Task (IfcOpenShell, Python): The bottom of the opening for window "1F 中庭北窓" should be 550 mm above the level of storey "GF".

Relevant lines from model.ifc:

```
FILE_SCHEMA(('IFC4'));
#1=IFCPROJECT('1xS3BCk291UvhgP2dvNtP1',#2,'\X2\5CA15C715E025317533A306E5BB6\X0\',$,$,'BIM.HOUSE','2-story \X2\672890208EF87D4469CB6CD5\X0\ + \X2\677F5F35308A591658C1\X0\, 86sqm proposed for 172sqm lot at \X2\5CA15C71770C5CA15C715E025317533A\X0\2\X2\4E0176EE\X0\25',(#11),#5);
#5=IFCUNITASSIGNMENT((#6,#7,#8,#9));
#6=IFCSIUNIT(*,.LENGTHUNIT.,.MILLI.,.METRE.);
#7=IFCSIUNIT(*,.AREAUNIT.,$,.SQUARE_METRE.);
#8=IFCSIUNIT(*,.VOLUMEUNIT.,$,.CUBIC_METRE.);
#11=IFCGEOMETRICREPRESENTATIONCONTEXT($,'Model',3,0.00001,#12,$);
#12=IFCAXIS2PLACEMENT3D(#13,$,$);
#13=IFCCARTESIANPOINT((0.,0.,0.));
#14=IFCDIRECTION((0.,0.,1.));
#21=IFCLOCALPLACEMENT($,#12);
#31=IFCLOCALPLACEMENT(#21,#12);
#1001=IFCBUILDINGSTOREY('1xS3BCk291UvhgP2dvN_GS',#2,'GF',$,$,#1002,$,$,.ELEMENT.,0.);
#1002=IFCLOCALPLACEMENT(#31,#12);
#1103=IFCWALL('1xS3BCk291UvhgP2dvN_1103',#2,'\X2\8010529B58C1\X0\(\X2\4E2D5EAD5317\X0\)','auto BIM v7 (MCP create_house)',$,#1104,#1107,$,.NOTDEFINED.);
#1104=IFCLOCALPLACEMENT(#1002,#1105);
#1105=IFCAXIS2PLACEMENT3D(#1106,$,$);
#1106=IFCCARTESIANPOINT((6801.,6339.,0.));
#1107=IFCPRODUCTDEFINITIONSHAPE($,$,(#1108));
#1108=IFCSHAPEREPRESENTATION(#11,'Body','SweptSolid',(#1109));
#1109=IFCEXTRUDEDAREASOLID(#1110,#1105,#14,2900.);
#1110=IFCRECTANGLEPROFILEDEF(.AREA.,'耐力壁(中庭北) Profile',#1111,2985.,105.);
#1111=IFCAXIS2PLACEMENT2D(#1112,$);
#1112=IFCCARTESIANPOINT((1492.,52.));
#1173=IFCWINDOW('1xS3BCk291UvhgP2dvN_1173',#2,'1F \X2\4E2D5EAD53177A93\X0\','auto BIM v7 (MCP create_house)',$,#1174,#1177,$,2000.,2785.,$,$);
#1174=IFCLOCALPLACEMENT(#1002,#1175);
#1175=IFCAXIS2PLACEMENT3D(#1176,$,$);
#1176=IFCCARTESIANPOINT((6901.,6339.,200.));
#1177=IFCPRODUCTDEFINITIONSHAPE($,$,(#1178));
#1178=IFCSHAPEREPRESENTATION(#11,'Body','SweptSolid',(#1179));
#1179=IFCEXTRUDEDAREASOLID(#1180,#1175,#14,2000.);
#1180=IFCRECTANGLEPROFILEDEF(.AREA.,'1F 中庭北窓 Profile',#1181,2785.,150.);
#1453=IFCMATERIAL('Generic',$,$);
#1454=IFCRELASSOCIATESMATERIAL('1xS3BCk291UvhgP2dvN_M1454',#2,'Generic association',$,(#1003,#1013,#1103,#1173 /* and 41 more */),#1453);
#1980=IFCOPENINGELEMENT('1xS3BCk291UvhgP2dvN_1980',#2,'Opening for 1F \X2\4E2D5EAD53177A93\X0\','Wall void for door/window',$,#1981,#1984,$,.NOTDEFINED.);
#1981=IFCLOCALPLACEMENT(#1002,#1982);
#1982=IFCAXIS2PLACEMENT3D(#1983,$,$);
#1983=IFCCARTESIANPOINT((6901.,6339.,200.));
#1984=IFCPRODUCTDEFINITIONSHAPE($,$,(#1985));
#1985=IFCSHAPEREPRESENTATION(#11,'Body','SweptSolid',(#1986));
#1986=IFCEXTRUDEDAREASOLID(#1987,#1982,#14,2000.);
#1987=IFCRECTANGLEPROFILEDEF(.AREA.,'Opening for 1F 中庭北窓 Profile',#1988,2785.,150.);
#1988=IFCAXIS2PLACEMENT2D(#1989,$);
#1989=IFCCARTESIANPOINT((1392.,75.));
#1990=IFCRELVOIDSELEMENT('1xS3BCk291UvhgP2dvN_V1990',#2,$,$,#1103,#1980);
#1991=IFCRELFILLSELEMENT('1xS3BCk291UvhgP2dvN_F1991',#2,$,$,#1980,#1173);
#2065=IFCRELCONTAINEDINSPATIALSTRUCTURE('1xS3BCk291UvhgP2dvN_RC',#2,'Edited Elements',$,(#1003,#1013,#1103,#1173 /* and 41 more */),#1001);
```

```python
import numpy as np
import ifcopenshell
import ifcopenshell.api.geometry
import ifcopenshell.geom
import ifcopenshell.util.element
import ifcopenshell.util.placement
import ifcopenshell.util.shape
import ifcopenshell.util.unit

model = ifcopenshell.open("model.ifc")
unit_scale = ifcopenshell.util.unit.calculate_unit_scale(model)

window = model.by_guid("1xS3BCk291UvhgP2dvN_1173")
opening = window.FillsVoids[0].RelatingOpeningElement
storey = ifcopenshell.util.element.get_container(window, ifc_class="IfcBuildingStorey")
level = ifcopenshell.util.placement.get_local_placement(storey.ObjectPlacement)[2, 3]

# The opening's origin need not be at the sill, so measure its lowest point.
shape = ifcopenshell.geom.create_shape(ifcopenshell.geom.settings(), opening)
bottom = ifcopenshell.util.shape.get_shape_bottom_elevation(shape, shape.geometry) / unit_scale
dz = level + 0.55 / unit_scale - bottom

shift = np.array([0.0, 0.0, dz])
# The window is not placed relative to its opening, so move both.
for product in (opening, window):
    matrix = ifcopenshell.util.placement.get_local_placement(product.ObjectPlacement)
    matrix[:3, 3] += shift
    ifcopenshell.api.geometry.edit_object_placement(model, product=product, matrix=matrix, is_si=False)

print(f"moved by {dz * unit_scale:+.3f} m")

model.write("model-out.ifc")
```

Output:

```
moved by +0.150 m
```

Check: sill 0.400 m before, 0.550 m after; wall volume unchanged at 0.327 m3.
